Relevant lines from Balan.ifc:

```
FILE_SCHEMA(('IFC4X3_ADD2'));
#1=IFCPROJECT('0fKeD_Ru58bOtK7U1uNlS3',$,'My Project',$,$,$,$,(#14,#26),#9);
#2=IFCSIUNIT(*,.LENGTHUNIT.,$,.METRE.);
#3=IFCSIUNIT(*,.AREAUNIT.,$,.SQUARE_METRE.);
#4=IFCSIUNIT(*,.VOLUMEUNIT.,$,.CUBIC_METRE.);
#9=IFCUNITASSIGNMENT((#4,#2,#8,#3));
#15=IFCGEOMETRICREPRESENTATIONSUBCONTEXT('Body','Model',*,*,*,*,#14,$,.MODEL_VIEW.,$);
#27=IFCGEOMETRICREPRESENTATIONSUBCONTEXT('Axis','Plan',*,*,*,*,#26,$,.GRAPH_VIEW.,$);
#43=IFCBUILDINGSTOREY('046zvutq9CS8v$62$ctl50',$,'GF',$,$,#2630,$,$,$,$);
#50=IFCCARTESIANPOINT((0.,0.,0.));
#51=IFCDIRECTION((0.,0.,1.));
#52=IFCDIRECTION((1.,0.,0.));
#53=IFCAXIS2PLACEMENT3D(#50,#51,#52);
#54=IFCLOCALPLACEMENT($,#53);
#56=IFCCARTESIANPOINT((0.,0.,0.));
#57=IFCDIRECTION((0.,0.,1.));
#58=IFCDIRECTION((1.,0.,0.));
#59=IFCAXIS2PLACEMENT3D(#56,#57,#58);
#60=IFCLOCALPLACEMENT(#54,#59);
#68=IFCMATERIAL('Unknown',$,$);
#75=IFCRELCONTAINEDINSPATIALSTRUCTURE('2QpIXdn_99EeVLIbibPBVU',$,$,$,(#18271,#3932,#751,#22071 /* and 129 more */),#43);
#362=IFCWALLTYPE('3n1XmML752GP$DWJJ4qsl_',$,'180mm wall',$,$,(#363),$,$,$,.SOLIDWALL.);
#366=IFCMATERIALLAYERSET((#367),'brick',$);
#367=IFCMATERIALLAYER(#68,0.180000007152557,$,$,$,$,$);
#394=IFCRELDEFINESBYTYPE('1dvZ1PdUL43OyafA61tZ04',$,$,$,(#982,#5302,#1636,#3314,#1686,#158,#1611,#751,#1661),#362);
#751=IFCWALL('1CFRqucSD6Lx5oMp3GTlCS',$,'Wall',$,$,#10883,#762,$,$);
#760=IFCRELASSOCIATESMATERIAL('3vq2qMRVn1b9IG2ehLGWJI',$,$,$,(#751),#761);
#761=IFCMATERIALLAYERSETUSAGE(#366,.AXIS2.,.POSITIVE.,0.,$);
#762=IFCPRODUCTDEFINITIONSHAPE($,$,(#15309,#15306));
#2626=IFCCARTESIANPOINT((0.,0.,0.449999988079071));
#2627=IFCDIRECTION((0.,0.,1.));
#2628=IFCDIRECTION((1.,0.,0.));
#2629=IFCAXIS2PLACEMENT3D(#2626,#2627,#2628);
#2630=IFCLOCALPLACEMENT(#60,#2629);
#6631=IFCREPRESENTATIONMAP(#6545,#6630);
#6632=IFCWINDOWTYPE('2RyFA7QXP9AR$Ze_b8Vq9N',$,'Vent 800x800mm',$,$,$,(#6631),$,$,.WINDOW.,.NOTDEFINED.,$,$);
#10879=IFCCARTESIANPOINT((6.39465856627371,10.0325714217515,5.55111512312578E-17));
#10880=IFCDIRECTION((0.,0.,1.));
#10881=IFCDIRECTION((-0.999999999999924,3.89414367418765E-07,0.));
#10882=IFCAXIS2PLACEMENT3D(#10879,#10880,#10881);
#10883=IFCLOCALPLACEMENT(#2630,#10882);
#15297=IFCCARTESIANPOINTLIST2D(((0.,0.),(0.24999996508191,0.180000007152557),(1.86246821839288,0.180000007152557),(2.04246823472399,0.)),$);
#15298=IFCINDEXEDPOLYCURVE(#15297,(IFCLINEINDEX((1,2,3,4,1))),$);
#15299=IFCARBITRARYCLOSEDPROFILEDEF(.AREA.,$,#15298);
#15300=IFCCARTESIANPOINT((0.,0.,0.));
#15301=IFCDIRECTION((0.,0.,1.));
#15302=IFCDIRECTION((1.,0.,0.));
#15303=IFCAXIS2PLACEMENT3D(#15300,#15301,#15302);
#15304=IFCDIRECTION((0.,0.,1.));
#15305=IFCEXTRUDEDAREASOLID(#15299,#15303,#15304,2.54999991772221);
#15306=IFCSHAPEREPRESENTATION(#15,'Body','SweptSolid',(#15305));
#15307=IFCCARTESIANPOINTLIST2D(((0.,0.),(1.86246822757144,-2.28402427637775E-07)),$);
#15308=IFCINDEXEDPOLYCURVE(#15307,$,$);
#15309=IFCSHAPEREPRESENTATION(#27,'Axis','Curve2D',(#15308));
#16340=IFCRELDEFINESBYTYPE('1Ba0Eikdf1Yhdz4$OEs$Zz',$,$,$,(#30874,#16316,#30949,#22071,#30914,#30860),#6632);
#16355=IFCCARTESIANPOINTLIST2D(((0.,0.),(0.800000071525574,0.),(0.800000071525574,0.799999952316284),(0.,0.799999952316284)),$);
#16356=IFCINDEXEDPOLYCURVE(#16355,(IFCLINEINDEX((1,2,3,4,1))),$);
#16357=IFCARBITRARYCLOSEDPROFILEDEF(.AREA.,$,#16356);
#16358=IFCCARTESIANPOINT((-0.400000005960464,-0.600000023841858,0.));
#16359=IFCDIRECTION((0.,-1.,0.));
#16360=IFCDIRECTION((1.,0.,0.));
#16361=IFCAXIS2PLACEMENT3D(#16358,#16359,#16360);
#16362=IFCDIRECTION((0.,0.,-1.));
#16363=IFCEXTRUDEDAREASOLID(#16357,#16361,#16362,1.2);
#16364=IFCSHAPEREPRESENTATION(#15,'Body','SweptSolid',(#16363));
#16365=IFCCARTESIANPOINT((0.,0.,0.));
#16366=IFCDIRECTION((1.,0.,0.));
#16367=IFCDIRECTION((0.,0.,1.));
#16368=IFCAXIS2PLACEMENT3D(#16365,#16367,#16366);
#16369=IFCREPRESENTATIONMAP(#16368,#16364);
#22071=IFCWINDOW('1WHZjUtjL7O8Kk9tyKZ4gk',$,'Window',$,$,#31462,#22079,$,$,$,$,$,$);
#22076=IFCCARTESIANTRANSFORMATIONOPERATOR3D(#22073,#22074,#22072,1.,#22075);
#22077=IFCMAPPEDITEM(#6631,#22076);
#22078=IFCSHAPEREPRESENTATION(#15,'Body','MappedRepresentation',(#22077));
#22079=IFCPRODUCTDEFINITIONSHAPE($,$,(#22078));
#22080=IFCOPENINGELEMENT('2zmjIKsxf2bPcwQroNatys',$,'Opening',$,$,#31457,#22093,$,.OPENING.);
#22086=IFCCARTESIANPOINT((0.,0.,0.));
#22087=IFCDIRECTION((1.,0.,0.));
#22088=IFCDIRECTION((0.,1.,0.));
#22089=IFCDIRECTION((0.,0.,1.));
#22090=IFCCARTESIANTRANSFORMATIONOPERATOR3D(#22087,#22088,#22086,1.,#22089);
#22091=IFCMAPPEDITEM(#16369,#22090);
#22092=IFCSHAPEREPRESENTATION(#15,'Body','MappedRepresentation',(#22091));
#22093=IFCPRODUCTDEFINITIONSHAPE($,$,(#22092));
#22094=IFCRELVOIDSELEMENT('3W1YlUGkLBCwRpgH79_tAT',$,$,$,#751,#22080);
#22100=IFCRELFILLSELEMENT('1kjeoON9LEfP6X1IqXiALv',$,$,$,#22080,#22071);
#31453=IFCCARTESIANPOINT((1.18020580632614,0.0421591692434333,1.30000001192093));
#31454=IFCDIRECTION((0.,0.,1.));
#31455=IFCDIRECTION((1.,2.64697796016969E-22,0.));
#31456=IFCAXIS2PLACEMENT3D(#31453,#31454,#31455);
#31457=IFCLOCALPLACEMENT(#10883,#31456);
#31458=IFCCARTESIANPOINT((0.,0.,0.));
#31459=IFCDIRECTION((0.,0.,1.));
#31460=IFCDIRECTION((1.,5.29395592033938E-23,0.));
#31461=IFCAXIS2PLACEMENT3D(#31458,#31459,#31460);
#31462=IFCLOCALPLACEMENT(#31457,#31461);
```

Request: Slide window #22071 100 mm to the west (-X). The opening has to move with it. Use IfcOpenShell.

```python
import ifcopenshell
import ifcopenshell.api.geometry
import ifcopenshell.util.placement
import ifcopenshell.util.unit

model = ifcopenshell.open("Balan.ifc")
unit_scale = ifcopenshell.util.unit.calculate_unit_scale(model)

window = model.by_guid("1WHZjUtjL7O8Kk9tyKZ4gk")
opening = window.FillsVoids[0].RelatingOpeningElement
wall = opening.VoidsElements[0].RelatingBuildingElement

wall_matrix = ifcopenshell.util.placement.get_local_placement(wall.ObjectPlacement)
shift = wall_matrix[:3, 0] * 0.1 / unit_scale
before = ifcopenshell.util.placement.get_local_placement(window.ObjectPlacement)[:3, 3].copy()

# The window is placed relative to its opening, so it follows when the opening moves.
matrix = ifcopenshell.util.placement.get_local_placement(opening.ObjectPlacement)
matrix[:3, 3] += shift
ifcopenshell.api.geometry.edit_object_placement(
    model, product=opening, matrix=matrix, is_si=False, should_transform_children=True
)

after = ifcopenshell.util.placement.get_local_placement(window.ObjectPlacement)[:3, 3]
print("window moved by", (after - before).round(3) + 0.0)

model.write("Balan_edited.ifc")
```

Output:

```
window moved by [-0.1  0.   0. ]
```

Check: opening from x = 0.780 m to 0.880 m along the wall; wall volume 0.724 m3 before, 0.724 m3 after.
